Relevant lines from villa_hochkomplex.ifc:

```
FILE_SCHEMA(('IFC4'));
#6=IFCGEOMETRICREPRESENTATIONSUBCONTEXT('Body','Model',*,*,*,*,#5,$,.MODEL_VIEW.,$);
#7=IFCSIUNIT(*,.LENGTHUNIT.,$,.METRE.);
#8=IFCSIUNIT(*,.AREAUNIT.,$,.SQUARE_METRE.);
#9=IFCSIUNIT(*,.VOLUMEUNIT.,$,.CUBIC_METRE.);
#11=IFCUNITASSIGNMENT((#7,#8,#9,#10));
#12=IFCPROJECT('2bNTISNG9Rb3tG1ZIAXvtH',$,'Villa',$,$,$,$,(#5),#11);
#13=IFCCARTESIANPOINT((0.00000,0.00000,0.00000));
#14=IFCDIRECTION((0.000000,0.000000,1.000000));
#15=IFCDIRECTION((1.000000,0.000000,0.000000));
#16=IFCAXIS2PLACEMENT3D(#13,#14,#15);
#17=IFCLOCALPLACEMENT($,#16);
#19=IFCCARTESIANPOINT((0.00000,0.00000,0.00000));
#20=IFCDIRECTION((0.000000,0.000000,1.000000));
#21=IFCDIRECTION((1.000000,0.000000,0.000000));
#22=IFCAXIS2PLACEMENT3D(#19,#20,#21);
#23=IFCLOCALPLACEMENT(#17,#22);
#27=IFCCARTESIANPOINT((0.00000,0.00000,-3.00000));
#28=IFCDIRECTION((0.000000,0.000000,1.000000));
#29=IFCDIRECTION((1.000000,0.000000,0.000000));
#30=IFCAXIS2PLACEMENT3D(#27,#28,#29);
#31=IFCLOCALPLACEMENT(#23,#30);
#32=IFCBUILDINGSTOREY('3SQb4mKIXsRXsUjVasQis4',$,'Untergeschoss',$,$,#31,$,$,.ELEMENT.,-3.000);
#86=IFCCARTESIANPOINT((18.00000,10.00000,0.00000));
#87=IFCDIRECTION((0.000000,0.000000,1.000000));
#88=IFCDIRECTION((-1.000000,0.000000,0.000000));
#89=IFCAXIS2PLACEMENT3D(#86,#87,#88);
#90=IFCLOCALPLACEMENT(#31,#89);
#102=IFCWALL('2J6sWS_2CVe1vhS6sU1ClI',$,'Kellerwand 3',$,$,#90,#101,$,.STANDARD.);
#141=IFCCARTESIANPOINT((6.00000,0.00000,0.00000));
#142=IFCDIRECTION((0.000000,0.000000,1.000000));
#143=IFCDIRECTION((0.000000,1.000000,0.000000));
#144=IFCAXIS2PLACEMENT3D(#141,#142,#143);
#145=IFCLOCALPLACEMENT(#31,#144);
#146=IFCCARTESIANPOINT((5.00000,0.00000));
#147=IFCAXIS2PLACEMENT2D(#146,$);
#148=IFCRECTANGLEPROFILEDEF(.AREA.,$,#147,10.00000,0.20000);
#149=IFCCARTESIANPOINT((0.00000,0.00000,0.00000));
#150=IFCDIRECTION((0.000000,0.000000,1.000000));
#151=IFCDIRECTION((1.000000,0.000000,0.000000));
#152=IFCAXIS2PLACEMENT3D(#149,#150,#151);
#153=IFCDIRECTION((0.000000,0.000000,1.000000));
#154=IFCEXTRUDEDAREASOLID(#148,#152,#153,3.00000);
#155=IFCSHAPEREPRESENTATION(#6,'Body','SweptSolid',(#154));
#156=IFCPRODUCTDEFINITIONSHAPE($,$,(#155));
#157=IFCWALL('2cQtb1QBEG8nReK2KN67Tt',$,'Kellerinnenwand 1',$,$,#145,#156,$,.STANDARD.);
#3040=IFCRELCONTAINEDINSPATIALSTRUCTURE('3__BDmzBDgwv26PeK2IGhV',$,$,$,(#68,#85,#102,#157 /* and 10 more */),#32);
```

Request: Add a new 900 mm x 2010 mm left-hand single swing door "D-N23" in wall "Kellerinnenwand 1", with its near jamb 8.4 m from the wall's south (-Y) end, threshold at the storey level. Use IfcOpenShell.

```python
import numpy as np
import ifcopenshell
import ifcopenshell.api.feature
import ifcopenshell.api.geometry
import ifcopenshell.api.root
import ifcopenshell.api.spatial
import ifcopenshell.geom
import ifcopenshell.util.element
import ifcopenshell.util.placement
import ifcopenshell.util.representation
import ifcopenshell.util.shape
import ifcopenshell.util.unit

model = ifcopenshell.open("villa_hochkomplex.ifc")
unit_scale = ifcopenshell.util.unit.calculate_unit_scale(model)
settings = ifcopenshell.geom.settings()


def volume(element):
    """Net volume in cubic metres, openings subtracted."""
    shape = ifcopenshell.geom.create_shape(settings, element)
    return ifcopenshell.util.shape.get_volume(shape.geometry)


wall = model.by_id(157)
storey = ifcopenshell.util.element.get_container(wall, ifc_class="IfcBuildingStorey")
context = ifcopenshell.util.representation.get_context(model, "Model", "Body", "MODEL_VIEW")
before = volume(wall)

width, height, from_end, sill = 0.9, 2.01, 8.4, 0.0  # metres

# The wall runs along its own X axis, and the end named is its -X end.
wall_shape = ifcopenshell.geom.create_shape(settings, wall)
x, y, z = ifcopenshell.util.shape.get_vertices(wall_shape.geometry).T
start = x.min() + from_end
face, thickness = float(y.min()), float(y.max() - y.min())
wall_matrix = ifcopenshell.util.placement.get_local_placement(wall.ObjectPlacement)
level = ifcopenshell.util.placement.get_local_placement(storey.ObjectPlacement)[2, 3]


def in_wall(x, y):
    """Placement at x, y metres in the wall's axes, at sill height."""
    matrix = wall_matrix.copy()
    matrix[:, 3] = wall_matrix @ np.array([x / unit_scale, y / unit_scale, 0.0, 1.0])
    matrix[2, 3] = level + sill / unit_scale
    return matrix


# Opening: a box that overshoots both wall faces by 50 mm.
opening = ifcopenshell.api.root.create_entity(model, ifc_class="IfcOpeningElement", predefined_type="OPENING")
box = ifcopenshell.api.geometry.add_wall_representation(
    model, context=context, length=width, height=height, thickness=thickness + 0.1
)
ifcopenshell.api.geometry.assign_representation(model, product=opening, representation=box)
ifcopenshell.api.geometry.edit_object_placement(model, product=opening, matrix=in_wall(start, face - 0.05), is_si=False)
ifcopenshell.api.feature.add_feature(model, feature=opening, element=wall)

door = ifcopenshell.api.root.create_entity(model, ifc_class="IfcDoor", name="D-N23", predefined_type="DOOR")
door.OverallWidth, door.OverallHeight = width / unit_scale, height / unit_scale
door.OperationType = "SINGLE_SWING_LEFT"
body = ifcopenshell.api.geometry.add_door_representation(
    model,
    context=context,
    overall_width=door.OverallWidth,
    overall_height=door.OverallHeight,
    operation_type="SINGLE_SWING_LEFT",
    lining_properties={"LiningDepth": thickness / unit_scale, "ThresholdDepth": thickness / unit_scale},
)
ifcopenshell.api.geometry.assign_representation(model, product=door, representation=body)
ifcopenshell.api.spatial.assign_container(model, products=[door], relating_structure=storey)
ifcopenshell.api.feature.add_filling(model, opening=opening, element=door)

# The lining spans the wall, so the door starts at the wall face.
ifcopenshell.api.geometry.edit_object_placement(model, product=door, matrix=in_wall(start, face), is_si=False)

after = volume(wall)

print(f"wall volume {before:.3f} -> {after:.3f} m3")

model.write("villa_hochkomplex_edited.ifc")
```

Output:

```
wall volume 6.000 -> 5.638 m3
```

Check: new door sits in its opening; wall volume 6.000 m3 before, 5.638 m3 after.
